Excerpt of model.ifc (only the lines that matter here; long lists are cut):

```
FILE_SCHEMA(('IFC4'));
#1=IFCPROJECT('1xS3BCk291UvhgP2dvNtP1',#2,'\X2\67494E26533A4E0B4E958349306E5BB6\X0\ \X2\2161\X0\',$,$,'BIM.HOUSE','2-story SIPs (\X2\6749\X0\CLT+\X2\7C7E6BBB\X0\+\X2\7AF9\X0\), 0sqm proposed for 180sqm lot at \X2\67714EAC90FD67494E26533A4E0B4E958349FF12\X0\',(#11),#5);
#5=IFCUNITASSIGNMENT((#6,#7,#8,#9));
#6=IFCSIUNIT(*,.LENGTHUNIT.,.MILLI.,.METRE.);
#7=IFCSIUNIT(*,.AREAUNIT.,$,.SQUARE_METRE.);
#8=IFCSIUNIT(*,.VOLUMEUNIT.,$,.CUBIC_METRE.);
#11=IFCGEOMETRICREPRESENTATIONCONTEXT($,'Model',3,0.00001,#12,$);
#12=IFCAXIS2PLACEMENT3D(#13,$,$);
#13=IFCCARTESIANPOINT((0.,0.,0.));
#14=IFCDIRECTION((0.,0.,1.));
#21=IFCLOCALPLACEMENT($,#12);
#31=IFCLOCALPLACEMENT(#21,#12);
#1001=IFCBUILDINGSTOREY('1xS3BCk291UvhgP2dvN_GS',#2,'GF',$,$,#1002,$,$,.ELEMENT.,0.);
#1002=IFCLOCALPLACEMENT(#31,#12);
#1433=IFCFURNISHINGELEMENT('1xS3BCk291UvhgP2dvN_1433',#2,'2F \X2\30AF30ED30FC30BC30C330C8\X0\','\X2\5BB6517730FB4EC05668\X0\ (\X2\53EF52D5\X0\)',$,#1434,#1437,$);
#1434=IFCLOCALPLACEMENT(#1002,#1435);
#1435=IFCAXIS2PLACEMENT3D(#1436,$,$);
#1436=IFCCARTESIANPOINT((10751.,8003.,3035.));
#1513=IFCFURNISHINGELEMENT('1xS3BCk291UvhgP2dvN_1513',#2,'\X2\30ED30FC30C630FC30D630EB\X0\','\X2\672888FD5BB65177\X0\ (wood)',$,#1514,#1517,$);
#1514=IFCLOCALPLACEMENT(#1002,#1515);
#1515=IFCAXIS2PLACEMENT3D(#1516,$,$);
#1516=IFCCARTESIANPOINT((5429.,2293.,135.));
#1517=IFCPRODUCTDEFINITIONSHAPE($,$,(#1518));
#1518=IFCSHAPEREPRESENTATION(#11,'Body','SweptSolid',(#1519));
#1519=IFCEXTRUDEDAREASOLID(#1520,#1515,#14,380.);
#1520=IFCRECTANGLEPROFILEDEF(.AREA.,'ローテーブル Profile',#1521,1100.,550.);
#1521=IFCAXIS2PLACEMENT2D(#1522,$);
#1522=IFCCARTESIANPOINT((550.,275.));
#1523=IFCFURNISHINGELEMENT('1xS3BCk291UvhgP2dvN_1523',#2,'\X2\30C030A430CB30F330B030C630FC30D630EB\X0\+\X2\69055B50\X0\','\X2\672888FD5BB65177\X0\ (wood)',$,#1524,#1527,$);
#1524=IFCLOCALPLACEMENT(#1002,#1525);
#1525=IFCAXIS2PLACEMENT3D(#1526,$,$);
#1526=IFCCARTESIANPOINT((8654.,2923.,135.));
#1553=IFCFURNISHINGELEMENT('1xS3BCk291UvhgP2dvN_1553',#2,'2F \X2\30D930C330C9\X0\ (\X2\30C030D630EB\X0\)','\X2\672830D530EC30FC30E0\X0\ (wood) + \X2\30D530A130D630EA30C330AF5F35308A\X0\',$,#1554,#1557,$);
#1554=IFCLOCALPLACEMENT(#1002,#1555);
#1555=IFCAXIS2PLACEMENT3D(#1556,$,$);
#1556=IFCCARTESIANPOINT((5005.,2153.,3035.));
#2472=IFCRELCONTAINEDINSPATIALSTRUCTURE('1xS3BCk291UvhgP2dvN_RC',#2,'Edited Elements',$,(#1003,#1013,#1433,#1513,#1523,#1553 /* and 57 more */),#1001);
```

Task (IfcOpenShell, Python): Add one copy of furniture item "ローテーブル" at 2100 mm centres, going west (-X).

```python
import numpy as np
import ifcopenshell
import ifcopenshell.api.geometry
import ifcopenshell.api.root
import ifcopenshell.util.element
import ifcopenshell.util.placement

model = ifcopenshell.open("model.ifc")


def reuse_history(source, copy):
    """copy_class also copies each property set's owner history, people and application; keep the originals."""
    for rel in copy.IsDefinedBy:
        if rel.is_a("IfcRelDefinesByProperties") and (history := rel.RelatingPropertyDefinition.OwnerHistory):
            rel.RelatingPropertyDefinition.OwnerHistory = source.OwnerHistory
            ifcopenshell.util.element.remove_deep2(model, history)


source = model.by_id(1513)
base = ifcopenshell.util.placement.get_local_placement(source.ObjectPlacement)
step = np.array([-1.0, 0.0, 0.0]) * 2100.0

for i in range(1, 2):
    copy = ifcopenshell.api.root.copy_class(model, product=source)
    copy.Representation = ifcopenshell.util.element.copy_deep(
        model, source.Representation, exclude=["IfcGeometricRepresentationContext", "IfcRepresentationMap"]
    )
    reuse_history(source, copy)
    matrix = base.copy()
    matrix[:3, 3] += i * step
    print("added at", matrix[:3, 3].round(3) + 0.0)
    ifcopenshell.api.geometry.edit_object_placement(model, product=copy, matrix=matrix, is_si=False)

model.write("model_v2.ifc")
```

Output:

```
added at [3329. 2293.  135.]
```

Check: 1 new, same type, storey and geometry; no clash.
